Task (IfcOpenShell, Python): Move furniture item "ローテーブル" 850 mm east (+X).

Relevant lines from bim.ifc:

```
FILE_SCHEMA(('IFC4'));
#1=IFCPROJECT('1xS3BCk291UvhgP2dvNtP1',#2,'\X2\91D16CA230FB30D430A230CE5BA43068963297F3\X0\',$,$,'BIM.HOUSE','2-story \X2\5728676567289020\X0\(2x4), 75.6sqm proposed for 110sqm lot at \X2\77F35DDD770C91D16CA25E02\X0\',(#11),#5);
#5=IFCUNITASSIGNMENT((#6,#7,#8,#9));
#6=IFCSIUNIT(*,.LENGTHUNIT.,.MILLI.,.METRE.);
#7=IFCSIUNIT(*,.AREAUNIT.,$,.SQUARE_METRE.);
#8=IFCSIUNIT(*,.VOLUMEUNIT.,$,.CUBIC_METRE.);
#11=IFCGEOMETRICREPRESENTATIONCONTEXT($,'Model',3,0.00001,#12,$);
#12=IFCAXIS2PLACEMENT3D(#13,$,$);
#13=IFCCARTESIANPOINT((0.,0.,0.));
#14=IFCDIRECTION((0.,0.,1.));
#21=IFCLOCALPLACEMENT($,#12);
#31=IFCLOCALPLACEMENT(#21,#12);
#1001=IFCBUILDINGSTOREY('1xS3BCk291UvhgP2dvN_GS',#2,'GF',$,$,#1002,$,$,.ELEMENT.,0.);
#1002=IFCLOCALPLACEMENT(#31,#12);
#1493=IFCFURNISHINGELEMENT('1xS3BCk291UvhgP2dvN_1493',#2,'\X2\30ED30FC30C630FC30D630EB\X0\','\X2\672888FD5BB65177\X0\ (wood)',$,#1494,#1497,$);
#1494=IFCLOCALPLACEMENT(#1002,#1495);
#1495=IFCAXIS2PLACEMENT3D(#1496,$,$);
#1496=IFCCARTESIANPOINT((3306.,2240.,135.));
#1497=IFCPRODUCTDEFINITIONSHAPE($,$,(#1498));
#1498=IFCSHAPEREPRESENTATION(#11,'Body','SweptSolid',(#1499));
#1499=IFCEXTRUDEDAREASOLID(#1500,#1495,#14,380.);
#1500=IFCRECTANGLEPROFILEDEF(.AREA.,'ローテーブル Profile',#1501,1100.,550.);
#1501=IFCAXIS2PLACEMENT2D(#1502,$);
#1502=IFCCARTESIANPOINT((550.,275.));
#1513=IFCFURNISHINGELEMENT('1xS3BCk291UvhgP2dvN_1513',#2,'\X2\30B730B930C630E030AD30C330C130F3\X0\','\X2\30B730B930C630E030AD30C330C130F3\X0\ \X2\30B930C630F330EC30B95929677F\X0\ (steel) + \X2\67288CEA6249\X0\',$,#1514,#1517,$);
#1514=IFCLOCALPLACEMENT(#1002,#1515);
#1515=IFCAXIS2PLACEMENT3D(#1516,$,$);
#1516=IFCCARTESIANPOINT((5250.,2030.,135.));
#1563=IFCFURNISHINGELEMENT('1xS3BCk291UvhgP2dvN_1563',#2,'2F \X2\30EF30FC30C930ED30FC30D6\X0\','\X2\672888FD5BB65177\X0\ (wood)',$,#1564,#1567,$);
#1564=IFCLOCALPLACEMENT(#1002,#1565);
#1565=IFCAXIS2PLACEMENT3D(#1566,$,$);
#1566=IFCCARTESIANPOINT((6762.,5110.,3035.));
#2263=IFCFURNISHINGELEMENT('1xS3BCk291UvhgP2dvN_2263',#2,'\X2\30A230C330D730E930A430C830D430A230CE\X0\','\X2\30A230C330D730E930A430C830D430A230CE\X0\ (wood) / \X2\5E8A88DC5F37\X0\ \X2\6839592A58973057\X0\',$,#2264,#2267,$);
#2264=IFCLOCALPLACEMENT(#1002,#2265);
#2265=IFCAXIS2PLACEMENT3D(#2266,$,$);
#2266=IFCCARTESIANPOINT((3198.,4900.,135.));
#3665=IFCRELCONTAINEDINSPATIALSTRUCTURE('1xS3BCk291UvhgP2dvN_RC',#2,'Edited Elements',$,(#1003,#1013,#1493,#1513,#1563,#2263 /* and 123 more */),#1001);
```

```python
import ifcopenshell
import ifcopenshell.api.geometry
import ifcopenshell.util.placement
import ifcopenshell.util.unit

model = ifcopenshell.open("bim.ifc")
unit_scale = ifcopenshell.util.unit.calculate_unit_scale(model)

item = model.by_guid("1xS3BCk291UvhgP2dvN_1493")
matrix = ifcopenshell.util.placement.get_local_placement(item.ObjectPlacement)
matrix[0, 3] += 0.85 / unit_scale
ifcopenshell.api.geometry.edit_object_placement(model, product=item, matrix=matrix, is_si=False)

print(ifcopenshell.util.placement.get_local_placement(item.ObjectPlacement).round(3) + 0.0)

model.write("bim_updated.ifc")
```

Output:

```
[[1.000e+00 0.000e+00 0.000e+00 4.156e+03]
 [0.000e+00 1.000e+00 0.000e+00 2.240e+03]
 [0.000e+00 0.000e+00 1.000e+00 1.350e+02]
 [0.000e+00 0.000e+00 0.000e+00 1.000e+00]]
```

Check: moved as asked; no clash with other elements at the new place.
